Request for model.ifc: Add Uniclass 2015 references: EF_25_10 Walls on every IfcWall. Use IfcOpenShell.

First a look at what the model holds.

```python
import ifcopenshell

model = ifcopenshell.open("model.ifc")
print(model.schema)
print("classifications:", [c.Name for c in model.by_type("IfcClassification")])
for ifc_class in ("IfcDoor", "IfcRoof", "IfcStair", "IfcWall", "IfcWindow"):
    print(ifc_class, len(model.by_type(ifc_class)))
```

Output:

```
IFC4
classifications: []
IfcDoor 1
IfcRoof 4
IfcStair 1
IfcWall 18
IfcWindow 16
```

```python
import ifcopenshell
import ifcopenshell.api.classification

model = ifcopenshell.open("model.ifc")

system = ifcopenshell.api.classification.add_classification(model, classification="Uniclass 2015")

codes = {
    "IfcWall": ("EF_25_10", "Walls"),
}
for ifc_class, (code, name) in codes.items():
    products = model.by_type(ifc_class)
    ifcopenshell.api.classification.add_reference(
        model, products=products, classification=system, identification=code, name=name
    )
    print(code, len(products))

model.write("model_edited.ifc")
```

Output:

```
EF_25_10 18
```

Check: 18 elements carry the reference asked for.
